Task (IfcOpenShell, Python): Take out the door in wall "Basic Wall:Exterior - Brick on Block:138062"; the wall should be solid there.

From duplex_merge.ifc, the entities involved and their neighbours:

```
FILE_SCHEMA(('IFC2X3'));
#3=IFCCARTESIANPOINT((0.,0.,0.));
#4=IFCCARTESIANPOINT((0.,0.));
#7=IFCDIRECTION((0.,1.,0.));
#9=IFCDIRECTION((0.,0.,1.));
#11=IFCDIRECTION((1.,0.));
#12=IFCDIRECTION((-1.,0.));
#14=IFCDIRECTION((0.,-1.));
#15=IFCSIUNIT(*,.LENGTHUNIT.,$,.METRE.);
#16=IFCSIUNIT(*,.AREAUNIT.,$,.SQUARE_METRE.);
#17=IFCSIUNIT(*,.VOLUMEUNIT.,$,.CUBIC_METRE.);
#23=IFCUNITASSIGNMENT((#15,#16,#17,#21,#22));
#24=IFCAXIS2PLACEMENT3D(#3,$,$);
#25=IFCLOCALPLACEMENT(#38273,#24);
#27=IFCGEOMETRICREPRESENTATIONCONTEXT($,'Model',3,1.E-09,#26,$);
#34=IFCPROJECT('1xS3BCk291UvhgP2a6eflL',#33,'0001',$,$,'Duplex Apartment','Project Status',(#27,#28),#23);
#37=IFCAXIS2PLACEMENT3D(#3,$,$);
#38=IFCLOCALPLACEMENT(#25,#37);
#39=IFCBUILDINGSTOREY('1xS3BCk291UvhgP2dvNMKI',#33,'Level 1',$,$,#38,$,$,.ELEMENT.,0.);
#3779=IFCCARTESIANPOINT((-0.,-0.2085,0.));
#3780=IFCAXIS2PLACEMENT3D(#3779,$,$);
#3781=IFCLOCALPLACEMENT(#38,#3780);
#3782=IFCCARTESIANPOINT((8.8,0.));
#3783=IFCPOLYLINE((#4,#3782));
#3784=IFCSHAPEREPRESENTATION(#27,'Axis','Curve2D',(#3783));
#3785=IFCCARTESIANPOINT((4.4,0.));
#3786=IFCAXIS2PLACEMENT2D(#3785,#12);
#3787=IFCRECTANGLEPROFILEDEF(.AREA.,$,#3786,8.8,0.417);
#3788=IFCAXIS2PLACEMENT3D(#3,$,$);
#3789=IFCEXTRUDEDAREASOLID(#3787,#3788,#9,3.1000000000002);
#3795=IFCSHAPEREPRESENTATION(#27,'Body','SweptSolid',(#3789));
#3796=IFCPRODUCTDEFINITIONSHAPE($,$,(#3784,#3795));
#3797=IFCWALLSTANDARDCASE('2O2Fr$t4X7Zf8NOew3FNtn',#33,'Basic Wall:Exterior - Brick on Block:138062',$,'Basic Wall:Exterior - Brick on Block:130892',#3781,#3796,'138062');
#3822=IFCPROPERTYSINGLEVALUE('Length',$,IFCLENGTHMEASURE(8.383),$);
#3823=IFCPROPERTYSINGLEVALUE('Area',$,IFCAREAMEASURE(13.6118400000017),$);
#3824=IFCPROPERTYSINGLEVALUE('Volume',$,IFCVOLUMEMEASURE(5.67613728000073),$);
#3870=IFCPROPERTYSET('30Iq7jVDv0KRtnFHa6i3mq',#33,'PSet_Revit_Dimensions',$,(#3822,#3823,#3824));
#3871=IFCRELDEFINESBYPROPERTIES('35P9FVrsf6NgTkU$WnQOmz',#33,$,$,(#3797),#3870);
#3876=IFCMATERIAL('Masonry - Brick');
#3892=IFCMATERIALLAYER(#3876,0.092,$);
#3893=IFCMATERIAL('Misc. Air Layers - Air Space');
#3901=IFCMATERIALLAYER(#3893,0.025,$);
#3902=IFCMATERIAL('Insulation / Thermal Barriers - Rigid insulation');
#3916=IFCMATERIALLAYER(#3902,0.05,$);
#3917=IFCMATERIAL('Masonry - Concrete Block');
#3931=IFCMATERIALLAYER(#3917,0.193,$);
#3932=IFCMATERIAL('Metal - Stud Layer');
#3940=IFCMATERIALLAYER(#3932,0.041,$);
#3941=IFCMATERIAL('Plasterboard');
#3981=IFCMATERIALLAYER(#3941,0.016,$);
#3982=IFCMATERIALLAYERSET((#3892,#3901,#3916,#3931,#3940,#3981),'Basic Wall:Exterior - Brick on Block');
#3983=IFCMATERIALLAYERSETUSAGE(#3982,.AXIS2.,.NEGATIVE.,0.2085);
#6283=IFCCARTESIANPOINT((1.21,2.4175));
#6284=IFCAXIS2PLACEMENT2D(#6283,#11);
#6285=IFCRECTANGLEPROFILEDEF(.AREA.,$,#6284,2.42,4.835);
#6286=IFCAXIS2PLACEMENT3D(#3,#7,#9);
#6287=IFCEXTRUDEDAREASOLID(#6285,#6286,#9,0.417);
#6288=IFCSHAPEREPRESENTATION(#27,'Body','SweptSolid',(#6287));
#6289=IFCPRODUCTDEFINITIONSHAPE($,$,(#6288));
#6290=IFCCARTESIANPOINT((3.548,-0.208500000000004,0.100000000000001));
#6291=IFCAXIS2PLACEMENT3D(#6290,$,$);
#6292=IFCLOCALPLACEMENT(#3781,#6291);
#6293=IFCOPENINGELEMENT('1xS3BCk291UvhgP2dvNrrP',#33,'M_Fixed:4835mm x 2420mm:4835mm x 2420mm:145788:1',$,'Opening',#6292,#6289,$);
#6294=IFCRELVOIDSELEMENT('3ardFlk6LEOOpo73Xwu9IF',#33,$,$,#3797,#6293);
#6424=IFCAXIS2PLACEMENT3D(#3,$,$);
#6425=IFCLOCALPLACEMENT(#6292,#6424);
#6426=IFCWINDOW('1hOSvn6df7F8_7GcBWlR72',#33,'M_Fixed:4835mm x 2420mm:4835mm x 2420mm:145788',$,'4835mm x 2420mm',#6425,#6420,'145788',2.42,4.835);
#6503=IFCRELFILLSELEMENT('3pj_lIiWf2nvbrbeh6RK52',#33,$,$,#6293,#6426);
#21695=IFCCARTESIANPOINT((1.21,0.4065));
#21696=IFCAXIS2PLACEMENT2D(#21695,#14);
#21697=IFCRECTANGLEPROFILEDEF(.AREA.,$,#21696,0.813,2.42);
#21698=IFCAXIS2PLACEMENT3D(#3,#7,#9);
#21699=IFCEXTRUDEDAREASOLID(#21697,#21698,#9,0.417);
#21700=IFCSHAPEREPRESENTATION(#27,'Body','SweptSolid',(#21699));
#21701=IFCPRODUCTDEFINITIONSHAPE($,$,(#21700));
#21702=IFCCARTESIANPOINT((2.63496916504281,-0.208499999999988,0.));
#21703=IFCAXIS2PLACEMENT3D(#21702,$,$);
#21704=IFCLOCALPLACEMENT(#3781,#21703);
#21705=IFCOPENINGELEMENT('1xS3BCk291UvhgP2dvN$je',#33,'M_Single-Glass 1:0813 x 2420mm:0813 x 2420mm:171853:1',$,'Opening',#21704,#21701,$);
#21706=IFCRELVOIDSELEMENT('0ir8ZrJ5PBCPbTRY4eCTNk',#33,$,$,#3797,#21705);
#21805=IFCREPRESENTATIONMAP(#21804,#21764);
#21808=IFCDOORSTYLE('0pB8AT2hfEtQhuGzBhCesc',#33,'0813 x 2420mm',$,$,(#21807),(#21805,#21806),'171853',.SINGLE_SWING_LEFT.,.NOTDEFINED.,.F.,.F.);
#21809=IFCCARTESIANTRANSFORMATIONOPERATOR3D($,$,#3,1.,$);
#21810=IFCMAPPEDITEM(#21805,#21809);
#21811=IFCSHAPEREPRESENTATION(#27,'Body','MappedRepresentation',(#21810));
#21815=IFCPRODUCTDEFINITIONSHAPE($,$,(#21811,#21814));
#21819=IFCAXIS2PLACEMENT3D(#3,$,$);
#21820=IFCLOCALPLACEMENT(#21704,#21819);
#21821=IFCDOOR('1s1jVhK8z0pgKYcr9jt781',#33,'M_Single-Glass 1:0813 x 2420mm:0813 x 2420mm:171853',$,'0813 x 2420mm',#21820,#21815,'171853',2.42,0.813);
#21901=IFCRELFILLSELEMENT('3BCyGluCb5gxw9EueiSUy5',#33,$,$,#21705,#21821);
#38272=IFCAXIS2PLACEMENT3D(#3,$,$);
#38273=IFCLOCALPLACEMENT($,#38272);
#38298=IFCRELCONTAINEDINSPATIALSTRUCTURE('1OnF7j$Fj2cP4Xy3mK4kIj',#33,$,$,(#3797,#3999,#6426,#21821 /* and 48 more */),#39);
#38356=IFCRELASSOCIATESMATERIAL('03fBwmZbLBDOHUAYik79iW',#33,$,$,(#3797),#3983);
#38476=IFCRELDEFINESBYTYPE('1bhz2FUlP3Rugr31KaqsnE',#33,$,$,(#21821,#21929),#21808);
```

```python
import ifcopenshell
import ifcopenshell.api.feature
import ifcopenshell.api.pset
import ifcopenshell.api.root
import ifcopenshell.geom
import ifcopenshell.util.element
import ifcopenshell.util.shape
import ifcopenshell.util.unit

model = ifcopenshell.open("duplex_merge.ifc")
area_scale = ifcopenshell.util.unit.calculate_unit_scale(model, "AREAUNIT")
volume_scale = ifcopenshell.util.unit.calculate_unit_scale(model, "VOLUMEUNIT")
settings = ifcopenshell.geom.settings()


def volume(element):
    """Net volume in cubic metres, openings subtracted."""
    shape = ifcopenshell.geom.create_shape(settings, element)
    return ifcopenshell.util.shape.get_volume(shape.geometry)


door = model.by_guid("1s1jVhK8z0pgKYcr9jt781")
opening = door.FillsVoids[0].RelatingOpeningElement
wall = opening.VoidsElements[0].RelatingBuildingElement
before = volume(wall)

ifcopenshell.api.root.remove_product(model, product=door)
ifcopenshell.api.feature.remove_feature(model, feature=opening)

after = volume(wall)
thickness = 0.417  # wall thickness in metres

# Update the wall's stored quantities.
pset = model.by_id(ifcopenshell.util.element.get_pset(wall, "PSet_Revit_Dimensions", should_inherit=False)["id"])
ifcopenshell.api.pset.edit_pset(model, pset=pset, properties={
    "Area": model.create_entity("IfcAreaMeasure", after / thickness / area_scale),
    "Volume": model.create_entity("IfcVolumeMeasure", after / volume_scale),
})

print(f"wall volume {before:.3f} -> {after:.3f} m3")

model.write("duplex_merge_rev.ifc")
```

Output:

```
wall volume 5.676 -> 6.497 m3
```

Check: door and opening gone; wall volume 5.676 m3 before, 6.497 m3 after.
